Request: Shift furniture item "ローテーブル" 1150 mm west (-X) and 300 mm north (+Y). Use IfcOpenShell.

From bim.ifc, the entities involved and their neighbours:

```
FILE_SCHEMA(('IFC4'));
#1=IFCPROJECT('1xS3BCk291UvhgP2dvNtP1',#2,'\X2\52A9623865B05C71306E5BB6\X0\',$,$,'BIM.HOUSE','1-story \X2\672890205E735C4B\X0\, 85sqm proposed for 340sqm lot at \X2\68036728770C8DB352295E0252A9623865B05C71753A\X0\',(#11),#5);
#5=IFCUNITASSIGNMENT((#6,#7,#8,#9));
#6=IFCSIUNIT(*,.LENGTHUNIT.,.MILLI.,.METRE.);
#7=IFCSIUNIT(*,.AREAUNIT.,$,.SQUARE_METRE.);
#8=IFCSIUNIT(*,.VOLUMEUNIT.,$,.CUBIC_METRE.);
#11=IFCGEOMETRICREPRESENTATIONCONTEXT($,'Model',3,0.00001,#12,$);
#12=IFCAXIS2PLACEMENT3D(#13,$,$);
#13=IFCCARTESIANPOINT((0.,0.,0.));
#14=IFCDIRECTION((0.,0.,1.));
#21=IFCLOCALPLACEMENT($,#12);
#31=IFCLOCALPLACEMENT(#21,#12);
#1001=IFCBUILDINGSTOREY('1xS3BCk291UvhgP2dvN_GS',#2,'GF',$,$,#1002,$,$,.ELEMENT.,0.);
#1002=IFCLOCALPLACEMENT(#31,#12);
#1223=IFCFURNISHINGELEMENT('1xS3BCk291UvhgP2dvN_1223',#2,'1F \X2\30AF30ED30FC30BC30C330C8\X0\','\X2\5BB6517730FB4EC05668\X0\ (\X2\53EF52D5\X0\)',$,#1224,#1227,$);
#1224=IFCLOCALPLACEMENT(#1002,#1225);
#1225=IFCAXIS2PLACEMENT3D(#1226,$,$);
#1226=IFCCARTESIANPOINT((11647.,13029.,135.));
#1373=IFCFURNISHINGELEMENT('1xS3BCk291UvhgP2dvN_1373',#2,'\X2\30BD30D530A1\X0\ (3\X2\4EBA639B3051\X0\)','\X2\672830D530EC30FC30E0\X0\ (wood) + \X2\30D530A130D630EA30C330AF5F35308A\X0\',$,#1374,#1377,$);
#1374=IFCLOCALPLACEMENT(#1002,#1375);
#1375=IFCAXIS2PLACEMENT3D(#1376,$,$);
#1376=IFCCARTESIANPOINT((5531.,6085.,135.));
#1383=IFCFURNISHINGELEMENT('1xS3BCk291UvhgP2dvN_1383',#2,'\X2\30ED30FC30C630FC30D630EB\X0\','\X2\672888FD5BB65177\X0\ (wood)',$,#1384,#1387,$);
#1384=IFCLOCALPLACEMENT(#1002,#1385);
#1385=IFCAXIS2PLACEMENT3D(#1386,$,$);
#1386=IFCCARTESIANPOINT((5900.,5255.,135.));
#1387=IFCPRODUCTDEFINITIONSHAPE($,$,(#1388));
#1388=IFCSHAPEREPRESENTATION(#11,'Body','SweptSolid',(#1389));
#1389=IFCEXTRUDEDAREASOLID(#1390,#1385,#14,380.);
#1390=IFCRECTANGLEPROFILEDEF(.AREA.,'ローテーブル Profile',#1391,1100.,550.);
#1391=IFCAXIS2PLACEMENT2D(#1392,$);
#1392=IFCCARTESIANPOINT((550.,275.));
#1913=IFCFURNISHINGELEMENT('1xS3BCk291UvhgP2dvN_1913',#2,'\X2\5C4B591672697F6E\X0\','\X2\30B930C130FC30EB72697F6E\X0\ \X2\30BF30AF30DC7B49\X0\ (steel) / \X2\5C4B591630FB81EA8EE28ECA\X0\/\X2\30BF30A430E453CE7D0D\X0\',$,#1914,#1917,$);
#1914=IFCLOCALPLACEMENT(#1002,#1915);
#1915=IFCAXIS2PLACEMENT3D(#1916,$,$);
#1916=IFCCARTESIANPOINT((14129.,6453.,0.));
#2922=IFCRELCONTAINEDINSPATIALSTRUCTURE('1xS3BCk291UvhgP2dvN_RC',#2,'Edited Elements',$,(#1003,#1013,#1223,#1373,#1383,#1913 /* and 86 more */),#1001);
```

```python
import ifcopenshell
import ifcopenshell.api.geometry
import ifcopenshell.util.placement

model = ifcopenshell.open("bim.ifc")

item = model.by_guid("1xS3BCk291UvhgP2dvN_1383")
matrix = ifcopenshell.util.placement.get_local_placement(item.ObjectPlacement)
matrix[0, 3] -= 1150.0
matrix[1, 3] += 300.0
ifcopenshell.api.geometry.edit_object_placement(model, product=item, matrix=matrix, is_si=False)

print(ifcopenshell.util.placement.get_local_placement(item.ObjectPlacement).round(3) + 0.0)

model.write("bim-out.ifc")
```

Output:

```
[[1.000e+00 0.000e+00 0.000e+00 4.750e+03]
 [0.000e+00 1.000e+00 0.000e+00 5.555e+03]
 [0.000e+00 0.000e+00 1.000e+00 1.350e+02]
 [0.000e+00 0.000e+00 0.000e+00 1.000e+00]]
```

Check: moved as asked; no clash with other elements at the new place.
